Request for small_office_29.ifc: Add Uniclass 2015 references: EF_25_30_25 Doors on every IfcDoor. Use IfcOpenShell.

First a look at what the model holds.

```python
import ifcopenshell

model = ifcopenshell.open("small_office_29.ifc")
print(model.schema)
print("classifications:", [c.Name for c in model.by_type("IfcClassification")])
for ifc_class in ("IfcDoor", "IfcRoof", "IfcStair", "IfcWall", "IfcWindow"):
    print(ifc_class, len(model.by_type(ifc_class)))
```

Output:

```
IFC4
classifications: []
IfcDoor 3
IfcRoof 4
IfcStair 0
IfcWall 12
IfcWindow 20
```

```python
import ifcopenshell
import ifcopenshell.api.classification

model = ifcopenshell.open("small_office_29.ifc")

system = ifcopenshell.api.classification.add_classification(model, classification="Uniclass 2015")

codes = {
    "IfcDoor": ("EF_25_30_25", "Doors"),
}
for ifc_class, (code, name) in codes.items():
    products = model.by_type(ifc_class)
    ifcopenshell.api.classification.add_reference(
        model, products=products, classification=system, identification=code, name=name
    )
    print(code, len(products))

model.write("small_office_29_v2.ifc")
```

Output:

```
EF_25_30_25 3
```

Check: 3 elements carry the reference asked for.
